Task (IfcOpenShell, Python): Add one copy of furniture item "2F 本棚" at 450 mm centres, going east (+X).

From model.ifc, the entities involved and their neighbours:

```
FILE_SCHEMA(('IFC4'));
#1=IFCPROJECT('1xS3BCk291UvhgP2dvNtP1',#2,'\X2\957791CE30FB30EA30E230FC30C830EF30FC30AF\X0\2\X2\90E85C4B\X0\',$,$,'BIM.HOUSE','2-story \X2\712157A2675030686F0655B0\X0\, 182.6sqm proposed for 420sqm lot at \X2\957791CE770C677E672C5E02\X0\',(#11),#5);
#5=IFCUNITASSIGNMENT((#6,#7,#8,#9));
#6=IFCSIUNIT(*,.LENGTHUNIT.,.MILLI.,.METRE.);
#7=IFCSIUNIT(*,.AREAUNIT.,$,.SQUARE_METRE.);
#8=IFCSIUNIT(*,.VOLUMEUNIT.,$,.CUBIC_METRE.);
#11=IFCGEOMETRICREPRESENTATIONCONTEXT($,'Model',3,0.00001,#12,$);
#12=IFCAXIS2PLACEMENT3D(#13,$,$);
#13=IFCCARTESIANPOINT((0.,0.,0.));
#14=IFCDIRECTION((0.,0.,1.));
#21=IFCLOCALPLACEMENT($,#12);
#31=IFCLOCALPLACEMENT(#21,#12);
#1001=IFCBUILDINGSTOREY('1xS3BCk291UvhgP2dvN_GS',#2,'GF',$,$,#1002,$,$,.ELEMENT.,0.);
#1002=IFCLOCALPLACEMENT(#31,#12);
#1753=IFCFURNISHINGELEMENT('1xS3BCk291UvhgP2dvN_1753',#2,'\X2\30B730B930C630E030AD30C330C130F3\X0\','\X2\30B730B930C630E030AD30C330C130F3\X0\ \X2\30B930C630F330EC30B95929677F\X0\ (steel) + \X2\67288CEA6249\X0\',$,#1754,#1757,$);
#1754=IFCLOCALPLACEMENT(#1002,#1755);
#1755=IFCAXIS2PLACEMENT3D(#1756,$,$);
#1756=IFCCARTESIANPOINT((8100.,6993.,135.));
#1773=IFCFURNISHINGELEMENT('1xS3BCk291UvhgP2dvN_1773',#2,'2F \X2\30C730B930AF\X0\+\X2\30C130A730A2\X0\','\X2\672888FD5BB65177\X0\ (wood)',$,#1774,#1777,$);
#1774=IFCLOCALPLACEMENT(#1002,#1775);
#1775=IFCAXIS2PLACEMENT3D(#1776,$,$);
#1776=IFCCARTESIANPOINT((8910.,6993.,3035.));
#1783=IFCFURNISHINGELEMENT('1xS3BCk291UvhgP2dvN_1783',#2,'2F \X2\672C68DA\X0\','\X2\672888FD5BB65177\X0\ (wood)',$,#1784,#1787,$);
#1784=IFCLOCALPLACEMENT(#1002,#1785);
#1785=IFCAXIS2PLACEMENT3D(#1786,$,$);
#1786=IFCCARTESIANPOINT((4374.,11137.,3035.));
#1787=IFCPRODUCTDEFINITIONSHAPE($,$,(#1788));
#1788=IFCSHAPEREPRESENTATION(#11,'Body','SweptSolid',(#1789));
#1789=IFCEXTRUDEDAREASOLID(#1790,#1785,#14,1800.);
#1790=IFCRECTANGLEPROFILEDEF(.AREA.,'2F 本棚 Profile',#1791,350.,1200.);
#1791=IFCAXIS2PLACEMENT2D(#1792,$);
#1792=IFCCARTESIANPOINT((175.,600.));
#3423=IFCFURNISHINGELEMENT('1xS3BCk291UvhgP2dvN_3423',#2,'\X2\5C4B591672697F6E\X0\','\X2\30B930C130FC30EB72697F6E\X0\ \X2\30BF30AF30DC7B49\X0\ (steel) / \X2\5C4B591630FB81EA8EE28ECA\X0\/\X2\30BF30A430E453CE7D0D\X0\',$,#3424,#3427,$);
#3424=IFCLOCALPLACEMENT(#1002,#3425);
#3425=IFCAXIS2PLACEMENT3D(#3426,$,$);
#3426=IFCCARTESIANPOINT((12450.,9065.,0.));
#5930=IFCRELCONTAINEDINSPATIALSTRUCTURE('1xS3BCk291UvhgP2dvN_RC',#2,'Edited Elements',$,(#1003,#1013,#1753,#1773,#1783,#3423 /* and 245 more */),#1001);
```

```python
import numpy as np
import ifcopenshell
import ifcopenshell.api.geometry
import ifcopenshell.api.root
import ifcopenshell.util.element
import ifcopenshell.util.placement
import ifcopenshell.util.unit

model = ifcopenshell.open("model.ifc")
unit_scale = ifcopenshell.util.unit.calculate_unit_scale(model)


def reuse_history(source, copy):
    """copy_class also copies each property set's owner history, people and application; keep the originals."""
    for rel in copy.IsDefinedBy:
        if rel.is_a("IfcRelDefinesByProperties") and (history := rel.RelatingPropertyDefinition.OwnerHistory):
            rel.RelatingPropertyDefinition.OwnerHistory = source.OwnerHistory
            ifcopenshell.util.element.remove_deep2(model, history)


source = model.by_guid("1xS3BCk291UvhgP2dvN_1783")
base = ifcopenshell.util.placement.get_local_placement(source.ObjectPlacement)
step = np.array([1.0, 0.0, 0.0]) * 0.45 / unit_scale

for i in range(1, 2):
    copy = ifcopenshell.api.root.copy_class(model, product=source)
    copy.Representation = ifcopenshell.util.element.copy_deep(
        model, source.Representation, exclude=["IfcGeometricRepresentationContext", "IfcRepresentationMap"]
    )
    reuse_history(source, copy)
    matrix = base.copy()
    matrix[:3, 3] += i * step
    print("added at", matrix[:3, 3].round(3) + 0.0)
    ifcopenshell.api.geometry.edit_object_placement(model, product=copy, matrix=matrix, is_si=False)

model.write("model_v2.ifc")
```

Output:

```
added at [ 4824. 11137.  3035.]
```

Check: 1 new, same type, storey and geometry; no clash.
